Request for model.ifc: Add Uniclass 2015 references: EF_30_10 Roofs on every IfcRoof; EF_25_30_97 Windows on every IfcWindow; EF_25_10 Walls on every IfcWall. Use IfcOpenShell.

First a look at what the model holds.

```python
import ifcopenshell

model = ifcopenshell.open("model.ifc")
print(model.schema)
print("classifications:", [c.Name for c in model.by_type("IfcClassification")])
for ifc_class in ("IfcDoor", "IfcRoof", "IfcStair", "IfcWall", "IfcWindow"):
    print(ifc_class, len(model.by_type(ifc_class)))
```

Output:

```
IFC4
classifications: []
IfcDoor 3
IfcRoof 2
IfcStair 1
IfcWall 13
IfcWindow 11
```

```python
import ifcopenshell
import ifcopenshell.api.classification

model = ifcopenshell.open("model.ifc")

system = ifcopenshell.api.classification.add_classification(model, classification="Uniclass 2015")

codes = {
    "IfcRoof": ("EF_30_10", "Roofs"),
    "IfcWindow": ("EF_25_30_97", "Windows"),
    "IfcWall": ("EF_25_10", "Walls"),
}
for ifc_class, (code, name) in codes.items():
    products = model.by_type(ifc_class)
    ifcopenshell.api.classification.add_reference(
        model, products=products, classification=system, identification=code, name=name
    )
    print(code, len(products))

model.write("model_v2.ifc")
```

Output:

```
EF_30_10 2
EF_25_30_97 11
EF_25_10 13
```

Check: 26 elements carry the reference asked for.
